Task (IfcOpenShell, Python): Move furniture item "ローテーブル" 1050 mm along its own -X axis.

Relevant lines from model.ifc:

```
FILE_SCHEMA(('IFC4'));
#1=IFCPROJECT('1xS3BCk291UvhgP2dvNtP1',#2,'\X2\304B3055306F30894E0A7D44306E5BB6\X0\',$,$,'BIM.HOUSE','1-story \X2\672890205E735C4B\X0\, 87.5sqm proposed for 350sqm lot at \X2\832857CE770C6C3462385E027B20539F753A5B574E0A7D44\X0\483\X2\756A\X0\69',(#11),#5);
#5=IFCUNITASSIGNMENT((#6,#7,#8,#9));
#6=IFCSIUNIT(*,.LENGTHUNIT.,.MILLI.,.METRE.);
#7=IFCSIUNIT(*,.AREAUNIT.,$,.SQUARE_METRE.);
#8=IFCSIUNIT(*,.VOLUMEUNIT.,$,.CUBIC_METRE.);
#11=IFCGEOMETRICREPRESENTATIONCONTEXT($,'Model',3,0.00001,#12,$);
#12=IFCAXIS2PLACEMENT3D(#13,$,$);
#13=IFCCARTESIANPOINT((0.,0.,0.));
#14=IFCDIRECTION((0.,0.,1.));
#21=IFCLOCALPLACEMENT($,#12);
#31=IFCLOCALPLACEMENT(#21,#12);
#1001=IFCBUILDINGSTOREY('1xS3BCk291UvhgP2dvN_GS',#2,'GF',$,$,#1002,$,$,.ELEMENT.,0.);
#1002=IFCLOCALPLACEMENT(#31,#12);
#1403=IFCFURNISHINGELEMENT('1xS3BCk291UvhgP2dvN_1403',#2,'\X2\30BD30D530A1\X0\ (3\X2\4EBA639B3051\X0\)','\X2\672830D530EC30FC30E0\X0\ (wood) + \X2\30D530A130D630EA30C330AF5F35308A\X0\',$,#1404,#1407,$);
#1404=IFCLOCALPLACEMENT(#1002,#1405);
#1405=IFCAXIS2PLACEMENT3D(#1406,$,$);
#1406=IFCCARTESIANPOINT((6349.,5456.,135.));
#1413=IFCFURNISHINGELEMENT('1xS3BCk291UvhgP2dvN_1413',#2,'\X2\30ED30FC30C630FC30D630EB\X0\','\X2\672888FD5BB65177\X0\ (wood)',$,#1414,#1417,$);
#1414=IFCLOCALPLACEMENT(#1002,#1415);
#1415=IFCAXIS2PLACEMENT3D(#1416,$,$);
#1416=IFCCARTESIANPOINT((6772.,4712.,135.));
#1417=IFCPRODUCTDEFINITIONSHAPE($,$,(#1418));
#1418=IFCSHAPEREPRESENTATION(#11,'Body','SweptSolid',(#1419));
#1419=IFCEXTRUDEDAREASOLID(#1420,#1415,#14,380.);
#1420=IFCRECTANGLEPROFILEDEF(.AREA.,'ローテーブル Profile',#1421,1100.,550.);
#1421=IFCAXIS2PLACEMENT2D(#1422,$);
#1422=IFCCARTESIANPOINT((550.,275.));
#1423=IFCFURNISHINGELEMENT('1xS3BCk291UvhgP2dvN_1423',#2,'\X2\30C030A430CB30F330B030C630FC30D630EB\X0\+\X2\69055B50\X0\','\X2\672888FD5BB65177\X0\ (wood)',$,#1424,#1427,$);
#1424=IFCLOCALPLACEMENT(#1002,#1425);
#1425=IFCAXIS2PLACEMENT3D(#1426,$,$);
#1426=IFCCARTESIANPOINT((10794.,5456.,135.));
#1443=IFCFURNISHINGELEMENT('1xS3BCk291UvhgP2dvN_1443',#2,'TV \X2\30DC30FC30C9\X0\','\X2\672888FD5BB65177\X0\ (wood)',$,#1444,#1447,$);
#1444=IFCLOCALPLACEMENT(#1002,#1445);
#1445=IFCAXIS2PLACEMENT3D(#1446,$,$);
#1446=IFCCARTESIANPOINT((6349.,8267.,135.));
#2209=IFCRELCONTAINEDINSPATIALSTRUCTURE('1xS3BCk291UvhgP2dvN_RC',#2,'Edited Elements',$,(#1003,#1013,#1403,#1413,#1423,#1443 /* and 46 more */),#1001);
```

```python
import ifcopenshell
import ifcopenshell.api.geometry
import ifcopenshell.util.placement
import ifcopenshell.util.unit

model = ifcopenshell.open("model.ifc")
unit_scale = ifcopenshell.util.unit.calculate_unit_scale(model)

item = model.by_guid("1xS3BCk291UvhgP2dvN_1413")
matrix = ifcopenshell.util.placement.get_local_placement(item.ObjectPlacement)
matrix[:3, 3] -= matrix[:3, 0] * 1.05 / unit_scale
ifcopenshell.api.geometry.edit_object_placement(model, product=item, matrix=matrix, is_si=False)

print(ifcopenshell.util.placement.get_local_placement(item.ObjectPlacement).round(3) + 0.0)

model.write("model_updated.ifc")
```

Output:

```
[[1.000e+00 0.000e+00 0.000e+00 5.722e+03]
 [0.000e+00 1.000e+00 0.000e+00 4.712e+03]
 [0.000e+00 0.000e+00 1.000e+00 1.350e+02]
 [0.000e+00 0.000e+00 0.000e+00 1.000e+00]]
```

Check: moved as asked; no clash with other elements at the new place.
